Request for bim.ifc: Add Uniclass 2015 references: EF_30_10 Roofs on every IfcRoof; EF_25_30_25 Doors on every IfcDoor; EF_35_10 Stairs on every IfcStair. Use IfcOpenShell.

First a look at what the model holds.

```python
import ifcopenshell

model = ifcopenshell.open("bim.ifc")
print(model.schema)
print("classifications:", [c.Name for c in model.by_type("IfcClassification")])
for ifc_class in ("IfcDoor", "IfcRoof", "IfcStair", "IfcWall", "IfcWindow"):
    print(ifc_class, len(model.by_type(ifc_class)))
```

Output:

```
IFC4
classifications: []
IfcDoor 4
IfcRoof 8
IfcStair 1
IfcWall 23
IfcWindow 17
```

```python
import ifcopenshell
import ifcopenshell.api.classification

model = ifcopenshell.open("bim.ifc")

system = ifcopenshell.api.classification.add_classification(model, classification="Uniclass 2015")

codes = {
    "IfcRoof": ("EF_30_10", "Roofs"),
    "IfcDoor": ("EF_25_30_25", "Doors"),
    "IfcStair": ("EF_35_10", "Stairs"),
}
for ifc_class, (code, name) in codes.items():
    products = model.by_type(ifc_class)
    ifcopenshell.api.classification.add_reference(
        model, products=products, classification=system, identification=code, name=name
    )
    print(code, len(products))

model.write("bim_updated.ifc")
```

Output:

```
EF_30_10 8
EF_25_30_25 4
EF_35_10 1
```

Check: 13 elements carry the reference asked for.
